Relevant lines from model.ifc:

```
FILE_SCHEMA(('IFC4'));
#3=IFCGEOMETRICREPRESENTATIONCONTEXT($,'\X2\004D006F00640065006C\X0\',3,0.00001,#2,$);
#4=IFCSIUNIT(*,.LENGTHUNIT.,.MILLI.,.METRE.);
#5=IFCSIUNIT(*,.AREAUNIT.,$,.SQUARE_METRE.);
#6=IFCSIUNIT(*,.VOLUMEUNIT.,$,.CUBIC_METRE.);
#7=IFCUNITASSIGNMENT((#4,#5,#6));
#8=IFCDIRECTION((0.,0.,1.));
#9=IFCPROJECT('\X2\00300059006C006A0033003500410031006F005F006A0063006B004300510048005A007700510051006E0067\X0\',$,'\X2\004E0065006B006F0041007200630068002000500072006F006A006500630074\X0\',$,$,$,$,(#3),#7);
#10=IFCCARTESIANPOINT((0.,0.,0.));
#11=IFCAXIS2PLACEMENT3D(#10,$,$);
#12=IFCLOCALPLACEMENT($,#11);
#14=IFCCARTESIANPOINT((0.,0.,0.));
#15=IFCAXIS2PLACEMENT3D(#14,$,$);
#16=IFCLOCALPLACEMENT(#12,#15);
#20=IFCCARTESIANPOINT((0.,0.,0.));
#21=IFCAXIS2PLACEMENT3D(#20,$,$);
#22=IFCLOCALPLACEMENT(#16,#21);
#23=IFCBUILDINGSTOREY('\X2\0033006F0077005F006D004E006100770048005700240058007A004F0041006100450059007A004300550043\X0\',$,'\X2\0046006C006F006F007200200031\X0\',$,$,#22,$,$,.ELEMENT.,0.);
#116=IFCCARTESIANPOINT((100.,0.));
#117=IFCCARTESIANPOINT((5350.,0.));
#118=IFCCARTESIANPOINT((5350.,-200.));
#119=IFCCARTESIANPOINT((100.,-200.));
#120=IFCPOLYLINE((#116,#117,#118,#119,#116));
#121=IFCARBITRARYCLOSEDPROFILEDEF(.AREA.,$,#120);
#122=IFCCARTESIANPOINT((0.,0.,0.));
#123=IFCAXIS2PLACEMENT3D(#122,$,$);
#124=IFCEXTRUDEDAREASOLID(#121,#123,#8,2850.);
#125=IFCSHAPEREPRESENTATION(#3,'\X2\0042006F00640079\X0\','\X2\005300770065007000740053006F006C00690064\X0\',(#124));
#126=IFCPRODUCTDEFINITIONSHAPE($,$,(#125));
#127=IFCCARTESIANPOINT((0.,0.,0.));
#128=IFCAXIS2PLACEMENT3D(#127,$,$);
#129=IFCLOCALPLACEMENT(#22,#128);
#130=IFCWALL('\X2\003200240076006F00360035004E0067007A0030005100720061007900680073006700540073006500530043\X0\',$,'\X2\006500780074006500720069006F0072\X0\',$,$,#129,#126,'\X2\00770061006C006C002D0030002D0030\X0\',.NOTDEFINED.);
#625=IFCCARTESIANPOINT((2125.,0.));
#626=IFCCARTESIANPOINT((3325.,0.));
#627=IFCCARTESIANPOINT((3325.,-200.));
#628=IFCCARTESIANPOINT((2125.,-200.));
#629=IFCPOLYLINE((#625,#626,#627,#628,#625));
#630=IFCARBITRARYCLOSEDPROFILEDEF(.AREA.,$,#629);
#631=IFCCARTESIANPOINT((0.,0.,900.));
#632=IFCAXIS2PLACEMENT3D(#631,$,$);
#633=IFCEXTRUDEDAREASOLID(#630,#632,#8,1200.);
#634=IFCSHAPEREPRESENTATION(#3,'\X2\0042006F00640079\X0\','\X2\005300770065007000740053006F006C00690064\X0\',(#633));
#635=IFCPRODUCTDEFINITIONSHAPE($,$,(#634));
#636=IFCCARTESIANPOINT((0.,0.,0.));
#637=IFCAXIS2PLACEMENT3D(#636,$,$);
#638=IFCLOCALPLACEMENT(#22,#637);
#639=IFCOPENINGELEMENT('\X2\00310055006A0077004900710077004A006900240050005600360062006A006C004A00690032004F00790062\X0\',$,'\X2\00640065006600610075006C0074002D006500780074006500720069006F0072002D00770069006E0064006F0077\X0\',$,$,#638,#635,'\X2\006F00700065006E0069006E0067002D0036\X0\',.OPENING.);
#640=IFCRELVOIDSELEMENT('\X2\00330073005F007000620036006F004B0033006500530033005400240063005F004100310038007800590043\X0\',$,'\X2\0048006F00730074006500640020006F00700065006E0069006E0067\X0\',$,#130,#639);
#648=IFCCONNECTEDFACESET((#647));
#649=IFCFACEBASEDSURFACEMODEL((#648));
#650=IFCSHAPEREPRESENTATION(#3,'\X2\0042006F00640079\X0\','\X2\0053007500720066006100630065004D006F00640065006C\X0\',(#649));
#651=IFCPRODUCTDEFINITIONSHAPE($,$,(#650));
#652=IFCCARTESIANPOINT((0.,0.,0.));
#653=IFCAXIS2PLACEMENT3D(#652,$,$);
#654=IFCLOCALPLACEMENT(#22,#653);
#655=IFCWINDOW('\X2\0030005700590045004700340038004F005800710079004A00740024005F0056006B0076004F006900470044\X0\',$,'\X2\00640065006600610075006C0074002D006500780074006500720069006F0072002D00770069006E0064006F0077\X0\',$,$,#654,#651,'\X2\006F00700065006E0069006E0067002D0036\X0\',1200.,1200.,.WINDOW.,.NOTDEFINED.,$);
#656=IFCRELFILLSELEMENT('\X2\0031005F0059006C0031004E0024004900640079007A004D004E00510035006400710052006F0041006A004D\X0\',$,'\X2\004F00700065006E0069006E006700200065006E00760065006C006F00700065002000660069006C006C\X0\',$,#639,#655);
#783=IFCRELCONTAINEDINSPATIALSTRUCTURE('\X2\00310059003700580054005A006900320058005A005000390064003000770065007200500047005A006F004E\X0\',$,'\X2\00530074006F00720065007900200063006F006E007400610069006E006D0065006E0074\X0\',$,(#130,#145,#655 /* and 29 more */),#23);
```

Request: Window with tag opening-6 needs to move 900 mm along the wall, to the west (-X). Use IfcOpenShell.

```python
import ifcopenshell
import ifcopenshell.api.geometry
import ifcopenshell.util.placement
import ifcopenshell.util.unit

model = ifcopenshell.open("model.ifc")
unit_scale = ifcopenshell.util.unit.calculate_unit_scale(model)

window = model.by_guid("0WYEG48OXqyJt$_VkvOiGD")
opening = window.FillsVoids[0].RelatingOpeningElement
wall = opening.VoidsElements[0].RelatingBuildingElement

wall_matrix = ifcopenshell.util.placement.get_local_placement(wall.ObjectPlacement)
shift = wall_matrix[:3, 0] * -0.9 / unit_scale
before = ifcopenshell.util.placement.get_local_placement(window.ObjectPlacement)[:3, 3].copy()

# The window is not placed relative to its opening, so move both.
for product in (opening, window):
    matrix = ifcopenshell.util.placement.get_local_placement(product.ObjectPlacement)
    matrix[:3, 3] += shift
    ifcopenshell.api.geometry.edit_object_placement(model, product=product, matrix=matrix, is_si=False)

after = ifcopenshell.util.placement.get_local_placement(window.ObjectPlacement)[:3, 3]
print("window moved by", (after - before).round(3) + 0.0)

model.write("model_rev.ifc")
```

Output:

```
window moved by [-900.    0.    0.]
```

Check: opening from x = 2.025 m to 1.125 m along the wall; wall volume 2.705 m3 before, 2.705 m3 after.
